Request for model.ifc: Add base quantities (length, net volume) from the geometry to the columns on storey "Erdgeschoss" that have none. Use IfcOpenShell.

First a look at what the model holds.

```python
import ifcopenshell
import ifcopenshell.util.element
import ifcopenshell.util.unit

model = ifcopenshell.open("model.ifc")
print(model.schema)
for unit_type in ("LENGTHUNIT", "AREAUNIT", "VOLUMEUNIT"):
    print(unit_type, ifcopenshell.util.unit.calculate_unit_scale(model, unit_type))
storey = next(s for s in model.by_type("IfcBuildingStorey") if s.Name == "Erdgeschoss")
columns = [e for e in ifcopenshell.util.element.get_decomposition(storey) if e.is_a("IfcColumn")]
for e in sorted(columns, key=lambda e: e.id()):
    print(e.id(), e.is_a(), e.Name, list(ifcopenshell.util.element.get_psets(e, qtos_only=True)), sep=" | ")
```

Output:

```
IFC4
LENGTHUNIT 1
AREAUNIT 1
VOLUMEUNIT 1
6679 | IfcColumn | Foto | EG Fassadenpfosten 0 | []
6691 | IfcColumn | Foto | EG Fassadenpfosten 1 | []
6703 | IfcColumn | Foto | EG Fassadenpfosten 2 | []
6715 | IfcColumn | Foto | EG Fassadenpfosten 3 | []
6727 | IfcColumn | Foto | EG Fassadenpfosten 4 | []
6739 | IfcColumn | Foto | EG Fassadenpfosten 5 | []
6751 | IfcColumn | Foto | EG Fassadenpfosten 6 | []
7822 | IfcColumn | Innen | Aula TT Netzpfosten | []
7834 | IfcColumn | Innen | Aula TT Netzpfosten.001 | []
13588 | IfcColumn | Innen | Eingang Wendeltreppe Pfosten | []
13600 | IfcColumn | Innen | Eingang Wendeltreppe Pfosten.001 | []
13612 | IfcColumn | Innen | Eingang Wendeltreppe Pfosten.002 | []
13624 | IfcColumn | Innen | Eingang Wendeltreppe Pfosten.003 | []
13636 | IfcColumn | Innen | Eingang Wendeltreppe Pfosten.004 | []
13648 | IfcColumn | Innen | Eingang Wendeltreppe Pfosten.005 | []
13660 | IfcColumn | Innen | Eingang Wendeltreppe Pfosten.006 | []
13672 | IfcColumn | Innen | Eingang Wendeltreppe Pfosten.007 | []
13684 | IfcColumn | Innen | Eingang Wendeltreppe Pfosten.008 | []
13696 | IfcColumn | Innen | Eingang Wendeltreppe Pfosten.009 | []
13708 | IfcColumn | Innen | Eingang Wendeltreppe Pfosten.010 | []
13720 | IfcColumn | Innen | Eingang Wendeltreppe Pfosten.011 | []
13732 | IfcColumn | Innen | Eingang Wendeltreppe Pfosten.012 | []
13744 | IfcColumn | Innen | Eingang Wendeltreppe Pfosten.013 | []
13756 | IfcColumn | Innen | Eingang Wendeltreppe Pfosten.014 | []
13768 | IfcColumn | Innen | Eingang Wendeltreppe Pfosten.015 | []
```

```python
import ifcopenshell
import ifcopenshell.api.pset
import ifcopenshell.geom
import ifcopenshell.util.element
import ifcopenshell.util.shape
import ifcopenshell.util.unit

model = ifcopenshell.open("model.ifc")
unit_scale = ifcopenshell.util.unit.calculate_unit_scale(model)
volume_scale = ifcopenshell.util.unit.calculate_unit_scale(model, "VOLUMEUNIT")
settings = ifcopenshell.geom.settings()

storey = next(s for s in model.by_type("IfcBuildingStorey") if s.Name == "Erdgeschoss")
columns = [e for e in ifcopenshell.util.element.get_decomposition(storey) if e.is_a("IfcColumn")]

for e in sorted(columns, key=lambda e: e.id()):
    if ifcopenshell.util.element.get_psets(e, qtos_only=True, should_inherit=False):
        continue
    # Geometry comes back in metres, in the element's own axes.
    shape = ifcopenshell.geom.create_shape(settings, e)
    values = {
        "Length": ifcopenshell.util.shape.get_z(shape.geometry) / unit_scale,
        "NetVolume": ifcopenshell.util.shape.get_volume(shape.geometry) / volume_scale,
    }
    qto = ifcopenshell.api.pset.add_qto(model, product=e, name="Qto_ColumnBaseQuantities")
    ifcopenshell.api.pset.edit_qto(model, qto=qto, properties=values)
    print(e.id(), {k: round(v, 3) for k, v in values.items()})

model.write("model-out.ifc")
```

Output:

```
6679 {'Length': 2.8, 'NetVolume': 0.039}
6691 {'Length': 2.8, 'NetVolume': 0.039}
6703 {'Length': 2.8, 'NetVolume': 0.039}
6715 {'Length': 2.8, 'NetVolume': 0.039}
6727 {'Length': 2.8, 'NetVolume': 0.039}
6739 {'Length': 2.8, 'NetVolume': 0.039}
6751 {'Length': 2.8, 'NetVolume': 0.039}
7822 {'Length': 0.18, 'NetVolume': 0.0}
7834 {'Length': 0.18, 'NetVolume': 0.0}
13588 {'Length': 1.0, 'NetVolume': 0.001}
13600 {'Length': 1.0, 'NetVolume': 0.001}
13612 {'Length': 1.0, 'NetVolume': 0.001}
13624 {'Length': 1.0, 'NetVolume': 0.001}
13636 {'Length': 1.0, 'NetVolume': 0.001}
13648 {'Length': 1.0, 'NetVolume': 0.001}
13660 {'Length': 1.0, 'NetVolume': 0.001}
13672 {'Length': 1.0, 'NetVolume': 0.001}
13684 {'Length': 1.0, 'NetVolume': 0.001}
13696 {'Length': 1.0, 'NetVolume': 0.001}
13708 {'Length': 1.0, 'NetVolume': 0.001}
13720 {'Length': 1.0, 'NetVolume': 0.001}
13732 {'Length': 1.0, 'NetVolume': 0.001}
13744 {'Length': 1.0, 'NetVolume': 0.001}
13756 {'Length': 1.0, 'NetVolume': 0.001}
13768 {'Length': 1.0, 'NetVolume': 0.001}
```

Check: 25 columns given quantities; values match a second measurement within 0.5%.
